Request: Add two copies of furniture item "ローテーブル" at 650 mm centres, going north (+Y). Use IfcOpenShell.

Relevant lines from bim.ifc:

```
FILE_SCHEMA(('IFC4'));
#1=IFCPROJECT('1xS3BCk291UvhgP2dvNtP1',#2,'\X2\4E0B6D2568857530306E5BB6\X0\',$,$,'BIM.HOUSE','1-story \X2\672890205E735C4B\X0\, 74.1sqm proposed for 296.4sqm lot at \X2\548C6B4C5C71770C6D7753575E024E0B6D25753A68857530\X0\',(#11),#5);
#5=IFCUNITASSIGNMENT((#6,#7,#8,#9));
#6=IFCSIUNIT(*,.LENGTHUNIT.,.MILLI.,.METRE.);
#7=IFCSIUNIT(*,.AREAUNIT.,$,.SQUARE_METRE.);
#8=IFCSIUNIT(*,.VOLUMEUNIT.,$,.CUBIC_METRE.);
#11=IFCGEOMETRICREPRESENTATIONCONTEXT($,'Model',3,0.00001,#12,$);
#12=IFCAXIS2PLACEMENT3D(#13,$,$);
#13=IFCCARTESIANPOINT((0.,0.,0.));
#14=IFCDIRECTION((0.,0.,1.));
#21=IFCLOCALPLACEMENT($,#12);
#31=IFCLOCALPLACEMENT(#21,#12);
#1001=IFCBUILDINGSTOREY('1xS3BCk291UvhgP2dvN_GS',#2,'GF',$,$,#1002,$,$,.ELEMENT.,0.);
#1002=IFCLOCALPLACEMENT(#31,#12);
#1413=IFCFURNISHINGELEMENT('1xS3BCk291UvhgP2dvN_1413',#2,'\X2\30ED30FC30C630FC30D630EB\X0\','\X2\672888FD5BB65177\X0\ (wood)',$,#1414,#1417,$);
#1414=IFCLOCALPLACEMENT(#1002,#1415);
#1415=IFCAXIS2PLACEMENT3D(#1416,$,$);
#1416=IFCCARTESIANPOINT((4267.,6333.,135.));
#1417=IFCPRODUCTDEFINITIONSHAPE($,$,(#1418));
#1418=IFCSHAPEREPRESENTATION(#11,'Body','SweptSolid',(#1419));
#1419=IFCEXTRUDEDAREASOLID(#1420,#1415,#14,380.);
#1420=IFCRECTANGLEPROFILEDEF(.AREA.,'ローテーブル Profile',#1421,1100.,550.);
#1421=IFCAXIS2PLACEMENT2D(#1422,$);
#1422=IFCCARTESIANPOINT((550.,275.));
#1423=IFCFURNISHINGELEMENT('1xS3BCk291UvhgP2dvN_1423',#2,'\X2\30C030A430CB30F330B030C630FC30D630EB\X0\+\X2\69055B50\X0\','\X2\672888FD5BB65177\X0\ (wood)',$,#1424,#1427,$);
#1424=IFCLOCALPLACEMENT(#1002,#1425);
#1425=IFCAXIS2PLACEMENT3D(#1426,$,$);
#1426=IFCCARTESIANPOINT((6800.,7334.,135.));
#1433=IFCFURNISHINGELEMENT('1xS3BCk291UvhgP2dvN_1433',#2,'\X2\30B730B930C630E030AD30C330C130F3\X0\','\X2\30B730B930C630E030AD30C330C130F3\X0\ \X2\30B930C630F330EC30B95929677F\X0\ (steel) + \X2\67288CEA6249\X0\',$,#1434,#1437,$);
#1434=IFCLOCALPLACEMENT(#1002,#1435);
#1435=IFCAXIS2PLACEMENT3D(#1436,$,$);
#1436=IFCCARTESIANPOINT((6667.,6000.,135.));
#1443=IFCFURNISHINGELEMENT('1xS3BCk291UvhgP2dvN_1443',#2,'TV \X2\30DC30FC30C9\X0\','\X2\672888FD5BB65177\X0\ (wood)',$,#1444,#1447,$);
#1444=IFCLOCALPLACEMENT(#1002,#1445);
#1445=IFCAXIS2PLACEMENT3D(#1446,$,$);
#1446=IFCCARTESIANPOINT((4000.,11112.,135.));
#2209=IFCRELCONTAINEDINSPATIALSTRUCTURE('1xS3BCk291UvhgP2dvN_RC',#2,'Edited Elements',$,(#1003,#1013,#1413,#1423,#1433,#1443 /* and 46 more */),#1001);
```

```python
import numpy as np
import ifcopenshell
import ifcopenshell.api.geometry
import ifcopenshell.api.root
import ifcopenshell.util.element
import ifcopenshell.util.placement

model = ifcopenshell.open("bim.ifc")


def reuse_history(source, copy):
    """copy_class also copies each property set's owner history, people and application; keep the originals."""
    for rel in copy.IsDefinedBy:
        if rel.is_a("IfcRelDefinesByProperties") and (history := rel.RelatingPropertyDefinition.OwnerHistory):
            rel.RelatingPropertyDefinition.OwnerHistory = source.OwnerHistory
            ifcopenshell.util.element.remove_deep2(model, history)


source = model.by_guid("1xS3BCk291UvhgP2dvN_1413")
base = ifcopenshell.util.placement.get_local_placement(source.ObjectPlacement)
step = np.array([0.0, 1.0, 0.0]) * 650.0

for i in range(1, 3):
    copy = ifcopenshell.api.root.copy_class(model, product=source)
    copy.Representation = ifcopenshell.util.element.copy_deep(
        model, source.Representation, exclude=["IfcGeometricRepresentationContext", "IfcRepresentationMap"]
    )
    reuse_history(source, copy)
    matrix = base.copy()
    matrix[:3, 3] += i * step
    print("added at", matrix[:3, 3].round(3) + 0.0)
    ifcopenshell.api.geometry.edit_object_placement(model, product=copy, matrix=matrix, is_si=False)

model.write("bim_edited.ifc")
```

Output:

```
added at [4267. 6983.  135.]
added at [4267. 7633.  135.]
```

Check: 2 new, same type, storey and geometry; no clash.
